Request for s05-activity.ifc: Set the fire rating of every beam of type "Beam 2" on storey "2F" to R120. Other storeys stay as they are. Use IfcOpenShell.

First a look at what the model holds.

```python
import ifcopenshell
import ifcopenshell.util.element

model = ifcopenshell.open("s05-activity.ifc")
print(model.schema)
storey = next(s for s in model.by_type("IfcBuildingStorey") if s.Name == "2F")
beams = [e for e in ifcopenshell.util.element.get_decomposition(storey) if e.is_a("IfcBeam")]
seen = {}
for e in beams:
    element_type = ifcopenshell.util.element.get_type(e)
    key = (element_type.Name if element_type != e and element_type else None, ifcopenshell.util.element.get_pset(e, "Pset_BeamCommon", "FireRating"))
    seen[key] = seen.get(key, 0) + 1
for (name, value), count in sorted(seen.items(), key=str):
    print(count, "x", name, "|", value)
```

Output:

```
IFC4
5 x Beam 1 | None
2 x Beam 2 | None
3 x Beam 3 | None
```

```python
import ifcopenshell
import ifcopenshell.api.pset
import ifcopenshell.util.element

model = ifcopenshell.open("s05-activity.ifc")

storey = next(s for s in model.by_type("IfcBuildingStorey") if s.Name == "2F")
beams = [e for e in ifcopenshell.util.element.get_decomposition(storey) if e.is_a("IfcBeam")]

count = 0
for e in beams:
    element_type = ifcopenshell.util.element.get_type(e)
    if element_type in (None, e) or element_type.Name != "Beam 2":
        continue
    # add_pset returns the element's existing set when there is one.
    pset = ifcopenshell.api.pset.add_pset(model, product=e, name="Pset_BeamCommon")
    ifcopenshell.api.pset.edit_pset(model, pset=pset, properties={"FireRating": "R120"})
    count += 1

print(count, "beams updated")

model.write("s05-activity_updated.ifc")
```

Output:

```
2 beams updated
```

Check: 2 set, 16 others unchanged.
